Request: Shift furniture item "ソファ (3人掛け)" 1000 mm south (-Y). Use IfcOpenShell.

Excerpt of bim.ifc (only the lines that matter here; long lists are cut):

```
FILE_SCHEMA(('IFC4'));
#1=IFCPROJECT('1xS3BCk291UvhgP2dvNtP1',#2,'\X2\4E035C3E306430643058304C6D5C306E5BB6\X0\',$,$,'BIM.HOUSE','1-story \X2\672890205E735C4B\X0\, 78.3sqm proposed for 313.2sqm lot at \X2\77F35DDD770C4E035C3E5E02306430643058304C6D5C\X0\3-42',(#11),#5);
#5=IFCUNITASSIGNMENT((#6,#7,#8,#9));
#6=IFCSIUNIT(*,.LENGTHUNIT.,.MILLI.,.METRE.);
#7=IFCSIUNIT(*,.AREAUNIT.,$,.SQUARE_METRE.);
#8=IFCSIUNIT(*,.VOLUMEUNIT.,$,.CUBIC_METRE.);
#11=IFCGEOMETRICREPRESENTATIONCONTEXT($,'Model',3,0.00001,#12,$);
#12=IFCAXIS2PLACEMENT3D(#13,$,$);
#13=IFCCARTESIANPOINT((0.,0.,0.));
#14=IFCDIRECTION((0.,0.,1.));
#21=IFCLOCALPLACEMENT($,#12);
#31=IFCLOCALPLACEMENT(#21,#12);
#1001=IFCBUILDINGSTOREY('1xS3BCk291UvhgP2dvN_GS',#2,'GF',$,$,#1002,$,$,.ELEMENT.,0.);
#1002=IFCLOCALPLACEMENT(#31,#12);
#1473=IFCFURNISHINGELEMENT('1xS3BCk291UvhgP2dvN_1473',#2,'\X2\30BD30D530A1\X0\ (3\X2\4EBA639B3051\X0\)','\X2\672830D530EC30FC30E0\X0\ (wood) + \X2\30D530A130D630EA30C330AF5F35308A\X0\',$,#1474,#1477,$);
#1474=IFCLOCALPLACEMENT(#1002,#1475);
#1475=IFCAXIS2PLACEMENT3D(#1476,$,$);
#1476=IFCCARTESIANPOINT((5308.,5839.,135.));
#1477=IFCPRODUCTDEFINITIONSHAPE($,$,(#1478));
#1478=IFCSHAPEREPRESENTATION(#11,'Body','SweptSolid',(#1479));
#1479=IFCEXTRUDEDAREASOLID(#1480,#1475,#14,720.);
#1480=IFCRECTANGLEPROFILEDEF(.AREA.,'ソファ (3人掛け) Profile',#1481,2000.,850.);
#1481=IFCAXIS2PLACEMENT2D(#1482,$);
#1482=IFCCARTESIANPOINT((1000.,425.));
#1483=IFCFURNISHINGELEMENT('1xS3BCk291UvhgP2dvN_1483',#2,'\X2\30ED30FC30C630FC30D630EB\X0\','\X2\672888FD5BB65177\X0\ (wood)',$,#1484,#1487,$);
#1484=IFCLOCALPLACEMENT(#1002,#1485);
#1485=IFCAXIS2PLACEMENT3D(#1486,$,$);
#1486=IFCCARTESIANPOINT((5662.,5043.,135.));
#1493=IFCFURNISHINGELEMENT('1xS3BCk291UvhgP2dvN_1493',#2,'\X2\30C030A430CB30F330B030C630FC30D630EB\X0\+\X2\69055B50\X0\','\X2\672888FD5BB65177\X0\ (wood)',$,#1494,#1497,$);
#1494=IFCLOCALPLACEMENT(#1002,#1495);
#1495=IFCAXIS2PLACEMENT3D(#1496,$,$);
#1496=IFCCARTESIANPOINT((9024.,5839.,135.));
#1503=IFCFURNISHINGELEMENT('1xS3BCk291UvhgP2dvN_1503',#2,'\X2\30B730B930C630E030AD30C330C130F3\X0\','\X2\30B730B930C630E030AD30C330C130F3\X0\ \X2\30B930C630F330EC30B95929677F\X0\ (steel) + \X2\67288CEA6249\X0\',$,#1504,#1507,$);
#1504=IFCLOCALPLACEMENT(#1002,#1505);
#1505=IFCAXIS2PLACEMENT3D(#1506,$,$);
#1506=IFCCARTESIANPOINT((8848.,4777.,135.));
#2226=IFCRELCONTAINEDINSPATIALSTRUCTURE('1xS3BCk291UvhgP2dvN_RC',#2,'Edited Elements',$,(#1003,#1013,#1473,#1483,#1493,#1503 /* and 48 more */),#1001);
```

```python
import ifcopenshell
import ifcopenshell.api.geometry
import ifcopenshell.util.placement

model = ifcopenshell.open("bim.ifc")

item = model.by_guid("1xS3BCk291UvhgP2dvN_1473")
matrix = ifcopenshell.util.placement.get_local_placement(item.ObjectPlacement)
matrix[1, 3] -= 1000.0
ifcopenshell.api.geometry.edit_object_placement(model, product=item, matrix=matrix, is_si=False)

print(ifcopenshell.util.placement.get_local_placement(item.ObjectPlacement).round(3) + 0.0)

model.write("bim_updated.ifc")
```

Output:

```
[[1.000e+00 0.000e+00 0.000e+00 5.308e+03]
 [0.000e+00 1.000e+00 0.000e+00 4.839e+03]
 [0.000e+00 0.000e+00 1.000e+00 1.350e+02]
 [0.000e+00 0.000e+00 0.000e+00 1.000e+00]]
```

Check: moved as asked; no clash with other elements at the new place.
